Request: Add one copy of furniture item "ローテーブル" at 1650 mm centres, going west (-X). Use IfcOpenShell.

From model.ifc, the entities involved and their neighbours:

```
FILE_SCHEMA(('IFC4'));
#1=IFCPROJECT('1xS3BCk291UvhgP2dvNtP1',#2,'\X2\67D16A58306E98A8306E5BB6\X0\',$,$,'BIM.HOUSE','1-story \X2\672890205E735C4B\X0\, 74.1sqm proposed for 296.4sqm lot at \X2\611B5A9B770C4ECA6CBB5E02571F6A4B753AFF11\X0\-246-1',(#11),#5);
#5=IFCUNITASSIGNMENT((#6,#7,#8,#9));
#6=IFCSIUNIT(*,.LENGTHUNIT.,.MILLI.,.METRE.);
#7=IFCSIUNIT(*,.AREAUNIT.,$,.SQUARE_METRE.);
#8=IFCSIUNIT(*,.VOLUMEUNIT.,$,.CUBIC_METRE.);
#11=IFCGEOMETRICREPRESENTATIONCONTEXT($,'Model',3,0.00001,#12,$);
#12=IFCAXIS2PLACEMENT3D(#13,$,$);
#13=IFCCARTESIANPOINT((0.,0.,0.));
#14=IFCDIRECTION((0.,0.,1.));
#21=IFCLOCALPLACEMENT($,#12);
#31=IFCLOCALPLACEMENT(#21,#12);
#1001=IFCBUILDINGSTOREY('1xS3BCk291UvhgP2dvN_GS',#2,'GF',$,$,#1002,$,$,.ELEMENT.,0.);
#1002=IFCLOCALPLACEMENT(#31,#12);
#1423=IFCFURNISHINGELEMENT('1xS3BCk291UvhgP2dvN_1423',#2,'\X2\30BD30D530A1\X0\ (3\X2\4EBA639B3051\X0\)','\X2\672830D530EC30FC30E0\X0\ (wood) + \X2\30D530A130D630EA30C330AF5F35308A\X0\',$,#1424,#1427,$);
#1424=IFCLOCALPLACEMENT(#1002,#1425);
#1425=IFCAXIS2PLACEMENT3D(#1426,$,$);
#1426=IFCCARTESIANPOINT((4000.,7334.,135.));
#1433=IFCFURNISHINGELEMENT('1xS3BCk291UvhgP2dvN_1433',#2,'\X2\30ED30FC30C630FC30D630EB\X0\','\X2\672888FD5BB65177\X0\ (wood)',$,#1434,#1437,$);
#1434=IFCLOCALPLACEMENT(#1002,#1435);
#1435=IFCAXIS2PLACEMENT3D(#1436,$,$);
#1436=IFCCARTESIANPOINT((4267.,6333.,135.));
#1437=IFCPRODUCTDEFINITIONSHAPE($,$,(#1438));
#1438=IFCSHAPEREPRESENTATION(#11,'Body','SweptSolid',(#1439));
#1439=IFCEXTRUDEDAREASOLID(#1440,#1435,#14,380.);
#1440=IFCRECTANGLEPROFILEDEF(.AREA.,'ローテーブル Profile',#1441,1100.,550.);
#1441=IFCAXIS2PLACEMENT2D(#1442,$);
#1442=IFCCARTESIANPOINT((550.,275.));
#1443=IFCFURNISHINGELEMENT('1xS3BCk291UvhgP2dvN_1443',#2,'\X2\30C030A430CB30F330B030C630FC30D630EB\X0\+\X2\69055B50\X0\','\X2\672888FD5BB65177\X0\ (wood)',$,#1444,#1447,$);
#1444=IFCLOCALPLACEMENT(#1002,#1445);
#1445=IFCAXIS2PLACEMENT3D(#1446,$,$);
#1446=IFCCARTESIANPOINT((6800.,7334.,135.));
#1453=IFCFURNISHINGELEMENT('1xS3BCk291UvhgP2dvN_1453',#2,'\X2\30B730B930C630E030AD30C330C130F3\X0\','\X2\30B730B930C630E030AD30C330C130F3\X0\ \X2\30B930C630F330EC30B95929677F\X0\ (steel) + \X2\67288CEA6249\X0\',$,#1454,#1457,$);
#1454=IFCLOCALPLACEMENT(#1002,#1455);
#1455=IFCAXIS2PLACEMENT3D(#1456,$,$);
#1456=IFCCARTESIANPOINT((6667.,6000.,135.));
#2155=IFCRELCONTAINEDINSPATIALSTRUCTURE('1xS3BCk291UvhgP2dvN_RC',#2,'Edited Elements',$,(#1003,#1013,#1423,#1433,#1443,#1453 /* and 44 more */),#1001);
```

```python
import numpy as np
import ifcopenshell
import ifcopenshell.api.geometry
import ifcopenshell.api.root
import ifcopenshell.util.element
import ifcopenshell.util.placement

model = ifcopenshell.open("model.ifc")


def reuse_history(source, copy):
    """copy_class also copies each property set's owner history, people and application; keep the originals."""
    for rel in copy.IsDefinedBy:
        if rel.is_a("IfcRelDefinesByProperties") and (history := rel.RelatingPropertyDefinition.OwnerHistory):
            rel.RelatingPropertyDefinition.OwnerHistory = source.OwnerHistory
            ifcopenshell.util.element.remove_deep2(model, history)


source = model.by_id(1433)
base = ifcopenshell.util.placement.get_local_placement(source.ObjectPlacement)
step = np.array([-1.0, 0.0, 0.0]) * 1650.0

for i in range(1, 2):
    copy = ifcopenshell.api.root.copy_class(model, product=source)
    copy.Representation = ifcopenshell.util.element.copy_deep(
        model, source.Representation, exclude=["IfcGeometricRepresentationContext", "IfcRepresentationMap"]
    )
    reuse_history(source, copy)
    matrix = base.copy()
    matrix[:3, 3] += i * step
    print("added at", matrix[:3, 3].round(3) + 0.0)
    ifcopenshell.api.geometry.edit_object_placement(model, product=copy, matrix=matrix, is_si=False)

model.write("model-out.ifc")
```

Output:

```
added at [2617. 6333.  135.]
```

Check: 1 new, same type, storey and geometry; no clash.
